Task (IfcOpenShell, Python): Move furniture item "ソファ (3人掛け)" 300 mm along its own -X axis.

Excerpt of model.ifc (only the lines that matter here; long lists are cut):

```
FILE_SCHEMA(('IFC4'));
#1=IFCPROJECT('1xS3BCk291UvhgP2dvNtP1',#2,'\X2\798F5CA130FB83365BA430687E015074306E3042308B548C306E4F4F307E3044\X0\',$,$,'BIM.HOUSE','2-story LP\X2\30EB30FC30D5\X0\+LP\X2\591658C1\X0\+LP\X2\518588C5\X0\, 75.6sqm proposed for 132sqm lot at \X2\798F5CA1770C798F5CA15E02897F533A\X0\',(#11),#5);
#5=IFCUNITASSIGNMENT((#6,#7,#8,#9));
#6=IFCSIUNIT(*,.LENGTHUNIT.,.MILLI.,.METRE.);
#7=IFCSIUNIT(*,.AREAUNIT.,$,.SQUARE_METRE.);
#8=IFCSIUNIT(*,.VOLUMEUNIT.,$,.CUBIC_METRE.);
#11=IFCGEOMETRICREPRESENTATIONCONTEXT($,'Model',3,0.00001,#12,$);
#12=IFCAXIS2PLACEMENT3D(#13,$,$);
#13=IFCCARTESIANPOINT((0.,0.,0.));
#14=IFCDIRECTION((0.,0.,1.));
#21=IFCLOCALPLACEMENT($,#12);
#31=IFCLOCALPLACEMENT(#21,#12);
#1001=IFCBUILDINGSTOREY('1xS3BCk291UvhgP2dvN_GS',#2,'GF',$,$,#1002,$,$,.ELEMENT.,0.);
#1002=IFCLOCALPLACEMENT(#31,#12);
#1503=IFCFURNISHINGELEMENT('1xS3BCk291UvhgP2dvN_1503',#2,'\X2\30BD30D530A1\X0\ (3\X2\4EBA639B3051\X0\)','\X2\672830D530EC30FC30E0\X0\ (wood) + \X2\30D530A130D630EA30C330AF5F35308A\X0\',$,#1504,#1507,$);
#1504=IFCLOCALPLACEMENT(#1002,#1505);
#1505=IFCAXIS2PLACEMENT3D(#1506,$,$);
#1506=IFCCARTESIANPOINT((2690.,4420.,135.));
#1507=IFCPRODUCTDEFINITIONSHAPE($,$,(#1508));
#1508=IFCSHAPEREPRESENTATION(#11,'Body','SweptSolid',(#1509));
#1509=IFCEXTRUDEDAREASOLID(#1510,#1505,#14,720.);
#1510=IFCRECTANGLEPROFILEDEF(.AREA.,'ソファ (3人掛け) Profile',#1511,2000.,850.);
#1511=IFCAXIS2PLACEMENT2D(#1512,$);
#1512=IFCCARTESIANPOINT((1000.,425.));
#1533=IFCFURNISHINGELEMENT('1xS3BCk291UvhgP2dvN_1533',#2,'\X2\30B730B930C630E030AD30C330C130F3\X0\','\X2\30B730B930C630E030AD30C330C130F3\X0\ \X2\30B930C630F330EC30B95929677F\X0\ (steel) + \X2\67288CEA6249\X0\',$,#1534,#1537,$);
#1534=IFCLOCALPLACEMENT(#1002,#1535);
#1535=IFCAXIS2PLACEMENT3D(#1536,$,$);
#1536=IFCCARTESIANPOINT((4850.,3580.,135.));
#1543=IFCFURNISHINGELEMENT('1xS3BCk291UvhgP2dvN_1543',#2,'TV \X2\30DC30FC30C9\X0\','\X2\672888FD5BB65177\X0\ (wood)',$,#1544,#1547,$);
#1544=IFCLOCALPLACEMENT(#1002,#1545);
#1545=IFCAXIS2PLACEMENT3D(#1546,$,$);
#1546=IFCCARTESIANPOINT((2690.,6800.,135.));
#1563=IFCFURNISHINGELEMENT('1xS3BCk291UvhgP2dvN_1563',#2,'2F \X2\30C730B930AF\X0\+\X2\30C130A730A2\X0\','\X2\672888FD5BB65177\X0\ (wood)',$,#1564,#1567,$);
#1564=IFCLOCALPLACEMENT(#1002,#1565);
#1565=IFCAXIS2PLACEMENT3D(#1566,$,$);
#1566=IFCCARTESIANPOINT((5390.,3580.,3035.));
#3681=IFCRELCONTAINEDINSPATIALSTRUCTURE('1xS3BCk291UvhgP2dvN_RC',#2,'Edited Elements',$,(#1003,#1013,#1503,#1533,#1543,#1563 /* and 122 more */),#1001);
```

```python
import ifcopenshell
import ifcopenshell.api.geometry
import ifcopenshell.util.placement
import ifcopenshell.util.unit

model = ifcopenshell.open("model.ifc")
unit_scale = ifcopenshell.util.unit.calculate_unit_scale(model)

item = model.by_id(1503)
matrix = ifcopenshell.util.placement.get_local_placement(item.ObjectPlacement)
matrix[:3, 3] -= matrix[:3, 0] * 0.3 / unit_scale
ifcopenshell.api.geometry.edit_object_placement(model, product=item, matrix=matrix, is_si=False)

print(ifcopenshell.util.placement.get_local_placement(item.ObjectPlacement).round(3) + 0.0)

model.write("model_edited.ifc")
```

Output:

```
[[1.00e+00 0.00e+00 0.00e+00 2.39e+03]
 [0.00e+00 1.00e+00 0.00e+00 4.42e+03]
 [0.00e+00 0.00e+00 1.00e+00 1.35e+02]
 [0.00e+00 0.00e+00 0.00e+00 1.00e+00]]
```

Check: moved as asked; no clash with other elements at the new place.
